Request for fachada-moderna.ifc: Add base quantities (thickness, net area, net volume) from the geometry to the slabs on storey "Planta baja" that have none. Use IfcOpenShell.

First a look at what the model holds.

```python
import ifcopenshell
import ifcopenshell.util.element
import ifcopenshell.util.unit

model = ifcopenshell.open("fachada-moderna.ifc")
print(model.schema)
for unit_type in ("LENGTHUNIT", "AREAUNIT", "VOLUMEUNIT"):
    print(unit_type, ifcopenshell.util.unit.calculate_unit_scale(model, unit_type))
storey = next(s for s in model.by_type("IfcBuildingStorey") if s.Name == "Planta baja")
slabs = [e for e in ifcopenshell.util.element.get_decomposition(storey) if e.is_a("IfcSlab")]
for e in sorted(slabs, key=lambda e: e.id()):
    print(e.id(), e.is_a(), e.Name, list(ifcopenshell.util.element.get_psets(e, qtos_only=True)), sep=" | ")
```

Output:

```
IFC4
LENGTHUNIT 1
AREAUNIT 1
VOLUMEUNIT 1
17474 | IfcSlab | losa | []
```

```python
import ifcopenshell
import ifcopenshell.api.pset
import ifcopenshell.geom
import ifcopenshell.util.element
import ifcopenshell.util.shape
import ifcopenshell.util.unit

model = ifcopenshell.open("fachada-moderna.ifc")
unit_scale = ifcopenshell.util.unit.calculate_unit_scale(model)
area_scale = ifcopenshell.util.unit.calculate_unit_scale(model, "AREAUNIT")
volume_scale = ifcopenshell.util.unit.calculate_unit_scale(model, "VOLUMEUNIT")
settings = ifcopenshell.geom.settings()

storey = next(s for s in model.by_type("IfcBuildingStorey") if s.Name == "Planta baja")
slabs = [e for e in ifcopenshell.util.element.get_decomposition(storey) if e.is_a("IfcSlab")]

for e in sorted(slabs, key=lambda e: e.id()):
    if ifcopenshell.util.element.get_psets(e, qtos_only=True, should_inherit=False):
        continue
    # Geometry comes back in metres, in the element's own axes.
    shape = ifcopenshell.geom.create_shape(settings, e)
    values = {
        "Width": ifcopenshell.util.shape.get_z(shape.geometry) / unit_scale,
        "NetArea": ifcopenshell.util.shape.get_footprint_area(shape.geometry) / area_scale,
        "NetVolume": ifcopenshell.util.shape.get_volume(shape.geometry) / volume_scale,
    }
    qto = ifcopenshell.api.pset.add_qto(model, product=e, name="Qto_SlabBaseQuantities")
    ifcopenshell.api.pset.edit_qto(model, qto=qto, properties=values)
    print(e.id(), {k: round(v, 3) for k, v in values.items()})

model.write("fachada-moderna_updated.ifc")
```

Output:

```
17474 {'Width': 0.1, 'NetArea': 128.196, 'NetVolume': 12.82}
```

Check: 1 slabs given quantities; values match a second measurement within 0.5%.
